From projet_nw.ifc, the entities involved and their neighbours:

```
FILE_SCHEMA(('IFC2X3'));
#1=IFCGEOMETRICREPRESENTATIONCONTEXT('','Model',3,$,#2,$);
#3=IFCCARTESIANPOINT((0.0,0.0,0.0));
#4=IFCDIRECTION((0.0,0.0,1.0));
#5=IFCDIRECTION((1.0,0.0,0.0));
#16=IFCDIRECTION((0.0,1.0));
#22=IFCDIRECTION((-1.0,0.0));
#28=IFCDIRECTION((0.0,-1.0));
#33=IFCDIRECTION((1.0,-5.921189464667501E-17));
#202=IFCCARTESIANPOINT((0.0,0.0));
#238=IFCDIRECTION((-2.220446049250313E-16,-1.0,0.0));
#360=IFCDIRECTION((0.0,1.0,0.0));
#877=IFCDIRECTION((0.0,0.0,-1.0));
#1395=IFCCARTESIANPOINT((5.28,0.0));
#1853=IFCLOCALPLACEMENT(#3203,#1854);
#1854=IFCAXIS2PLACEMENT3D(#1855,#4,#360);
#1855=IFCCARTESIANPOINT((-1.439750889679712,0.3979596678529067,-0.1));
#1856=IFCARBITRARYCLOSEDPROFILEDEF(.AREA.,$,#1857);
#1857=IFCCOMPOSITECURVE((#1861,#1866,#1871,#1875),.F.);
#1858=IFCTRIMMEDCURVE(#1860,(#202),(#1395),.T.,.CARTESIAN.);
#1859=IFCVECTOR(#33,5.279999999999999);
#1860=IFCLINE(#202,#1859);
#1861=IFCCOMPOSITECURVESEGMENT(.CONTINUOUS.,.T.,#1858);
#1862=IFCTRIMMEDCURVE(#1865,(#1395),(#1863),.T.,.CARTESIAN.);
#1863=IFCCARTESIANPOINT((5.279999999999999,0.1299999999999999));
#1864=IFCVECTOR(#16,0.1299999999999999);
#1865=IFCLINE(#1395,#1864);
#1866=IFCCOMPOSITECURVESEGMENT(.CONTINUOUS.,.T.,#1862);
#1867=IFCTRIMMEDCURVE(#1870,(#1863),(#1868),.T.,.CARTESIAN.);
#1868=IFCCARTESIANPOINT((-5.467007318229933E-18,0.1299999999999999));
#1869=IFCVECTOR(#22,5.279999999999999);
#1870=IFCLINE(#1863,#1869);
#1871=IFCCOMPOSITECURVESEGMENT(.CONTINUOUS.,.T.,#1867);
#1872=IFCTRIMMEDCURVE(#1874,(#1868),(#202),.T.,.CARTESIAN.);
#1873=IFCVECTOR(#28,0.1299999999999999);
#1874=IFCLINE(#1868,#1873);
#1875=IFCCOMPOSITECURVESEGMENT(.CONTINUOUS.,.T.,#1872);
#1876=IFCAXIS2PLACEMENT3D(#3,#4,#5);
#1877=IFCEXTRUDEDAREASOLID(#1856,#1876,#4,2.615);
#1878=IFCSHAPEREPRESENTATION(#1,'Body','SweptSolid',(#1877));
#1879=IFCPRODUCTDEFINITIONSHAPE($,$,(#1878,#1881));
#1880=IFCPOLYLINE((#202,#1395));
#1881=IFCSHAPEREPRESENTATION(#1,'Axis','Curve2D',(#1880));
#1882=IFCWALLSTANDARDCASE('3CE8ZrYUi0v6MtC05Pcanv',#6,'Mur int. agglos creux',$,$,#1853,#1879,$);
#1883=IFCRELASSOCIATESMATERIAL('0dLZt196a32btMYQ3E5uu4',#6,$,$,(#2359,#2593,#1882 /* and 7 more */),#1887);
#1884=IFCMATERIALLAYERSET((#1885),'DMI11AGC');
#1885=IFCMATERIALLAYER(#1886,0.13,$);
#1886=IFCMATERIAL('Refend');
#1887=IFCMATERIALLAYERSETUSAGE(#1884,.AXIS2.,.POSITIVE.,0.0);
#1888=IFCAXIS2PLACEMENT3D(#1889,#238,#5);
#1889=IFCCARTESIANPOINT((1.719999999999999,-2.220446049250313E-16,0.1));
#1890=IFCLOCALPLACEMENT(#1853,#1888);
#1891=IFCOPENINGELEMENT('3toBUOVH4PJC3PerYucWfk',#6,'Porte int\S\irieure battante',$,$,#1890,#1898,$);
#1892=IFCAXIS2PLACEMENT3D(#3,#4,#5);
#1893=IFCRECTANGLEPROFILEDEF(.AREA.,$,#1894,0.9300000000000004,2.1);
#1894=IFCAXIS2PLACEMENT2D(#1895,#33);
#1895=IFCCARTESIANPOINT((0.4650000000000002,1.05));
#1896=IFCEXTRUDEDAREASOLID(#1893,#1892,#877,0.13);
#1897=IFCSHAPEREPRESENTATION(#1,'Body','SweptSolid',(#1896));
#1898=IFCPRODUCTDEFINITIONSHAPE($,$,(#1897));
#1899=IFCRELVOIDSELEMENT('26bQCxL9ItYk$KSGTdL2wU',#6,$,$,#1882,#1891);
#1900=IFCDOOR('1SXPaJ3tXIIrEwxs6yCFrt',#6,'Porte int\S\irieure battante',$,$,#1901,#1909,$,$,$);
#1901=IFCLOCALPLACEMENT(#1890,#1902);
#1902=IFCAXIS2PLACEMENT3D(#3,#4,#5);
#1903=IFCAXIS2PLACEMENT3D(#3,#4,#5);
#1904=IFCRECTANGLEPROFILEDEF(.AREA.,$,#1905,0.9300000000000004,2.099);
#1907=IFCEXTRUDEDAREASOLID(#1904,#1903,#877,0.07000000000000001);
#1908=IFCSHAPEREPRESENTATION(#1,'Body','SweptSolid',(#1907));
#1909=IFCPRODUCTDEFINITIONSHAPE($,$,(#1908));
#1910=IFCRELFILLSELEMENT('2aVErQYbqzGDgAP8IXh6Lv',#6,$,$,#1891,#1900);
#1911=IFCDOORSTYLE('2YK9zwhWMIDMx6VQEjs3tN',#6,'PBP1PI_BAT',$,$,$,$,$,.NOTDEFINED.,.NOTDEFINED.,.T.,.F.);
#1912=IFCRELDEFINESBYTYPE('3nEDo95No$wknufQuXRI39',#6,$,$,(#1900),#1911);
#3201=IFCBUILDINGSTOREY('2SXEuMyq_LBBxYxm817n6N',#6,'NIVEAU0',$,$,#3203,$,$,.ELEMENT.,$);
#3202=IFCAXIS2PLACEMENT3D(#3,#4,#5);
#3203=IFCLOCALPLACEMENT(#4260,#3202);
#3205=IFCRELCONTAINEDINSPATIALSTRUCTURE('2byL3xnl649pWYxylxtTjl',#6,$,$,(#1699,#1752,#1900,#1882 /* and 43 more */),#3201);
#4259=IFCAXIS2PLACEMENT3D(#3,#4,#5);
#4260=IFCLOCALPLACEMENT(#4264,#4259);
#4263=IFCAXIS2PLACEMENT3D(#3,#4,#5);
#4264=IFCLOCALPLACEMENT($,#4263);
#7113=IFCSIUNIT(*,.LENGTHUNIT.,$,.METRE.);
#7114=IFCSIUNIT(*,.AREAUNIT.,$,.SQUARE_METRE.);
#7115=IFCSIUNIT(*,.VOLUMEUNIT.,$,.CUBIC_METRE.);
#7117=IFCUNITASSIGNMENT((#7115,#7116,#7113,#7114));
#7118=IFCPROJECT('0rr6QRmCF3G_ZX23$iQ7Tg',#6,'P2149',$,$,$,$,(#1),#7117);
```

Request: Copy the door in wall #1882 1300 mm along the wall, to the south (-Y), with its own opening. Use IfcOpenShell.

```python
import ifcopenshell
import ifcopenshell.api.feature
import ifcopenshell.api.geometry
import ifcopenshell.api.root
import ifcopenshell.geom
import ifcopenshell.util.element
import ifcopenshell.util.placement
import ifcopenshell.util.shape
import ifcopenshell.util.unit

model = ifcopenshell.open("projet_nw.ifc")
unit_scale = ifcopenshell.util.unit.calculate_unit_scale(model)
settings = ifcopenshell.geom.settings()


def volume(element):
    """Net volume in cubic metres, openings subtracted."""
    shape = ifcopenshell.geom.create_shape(settings, element)
    return ifcopenshell.util.shape.get_volume(shape.geometry)


door = model.by_guid("1SXPaJ3tXIIrEwxs6yCFrt")
opening = door.FillsVoids[0].RelatingOpeningElement
wall = opening.VoidsElements[0].RelatingBuildingElement
before = volume(wall)
shift = ifcopenshell.util.placement.get_local_placement(wall.ObjectPlacement)[:3, 0] * -1.3 / unit_scale

# copy_class copies the void relationship, type, container and properties, but no geometry.
new_opening = ifcopenshell.api.root.copy_class(model, product=opening)
new_opening.Representation = ifcopenshell.util.element.copy_deep(
    model, opening.Representation, exclude=["IfcGeometricRepresentationContext", "IfcRepresentationMap"]
)
new_door = ifcopenshell.api.root.copy_class(model, product=door)
new_door.Representation = ifcopenshell.util.element.copy_deep(
    model, door.Representation, exclude=["IfcGeometricRepresentationContext", "IfcRepresentationMap"]
)
fills = ifcopenshell.api.feature.add_filling(model, opening=new_opening, element=new_door)
fills.OwnerHistory = new_door.OwnerHistory  # required in IFC2X3

for old, new in ((opening, new_opening), (door, new_door)):
    matrix = ifcopenshell.util.placement.get_local_placement(old.ObjectPlacement)
    matrix[:3, 3] += shift
    ifcopenshell.api.geometry.edit_object_placement(model, product=new, matrix=matrix, is_si=False)

after = volume(wall)

print(f"wall volume {before:.3f} -> {after:.3f} m3")

model.write("projet_nw_edited.ifc")
```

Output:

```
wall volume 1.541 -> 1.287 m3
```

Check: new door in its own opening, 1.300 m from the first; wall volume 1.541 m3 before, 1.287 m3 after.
